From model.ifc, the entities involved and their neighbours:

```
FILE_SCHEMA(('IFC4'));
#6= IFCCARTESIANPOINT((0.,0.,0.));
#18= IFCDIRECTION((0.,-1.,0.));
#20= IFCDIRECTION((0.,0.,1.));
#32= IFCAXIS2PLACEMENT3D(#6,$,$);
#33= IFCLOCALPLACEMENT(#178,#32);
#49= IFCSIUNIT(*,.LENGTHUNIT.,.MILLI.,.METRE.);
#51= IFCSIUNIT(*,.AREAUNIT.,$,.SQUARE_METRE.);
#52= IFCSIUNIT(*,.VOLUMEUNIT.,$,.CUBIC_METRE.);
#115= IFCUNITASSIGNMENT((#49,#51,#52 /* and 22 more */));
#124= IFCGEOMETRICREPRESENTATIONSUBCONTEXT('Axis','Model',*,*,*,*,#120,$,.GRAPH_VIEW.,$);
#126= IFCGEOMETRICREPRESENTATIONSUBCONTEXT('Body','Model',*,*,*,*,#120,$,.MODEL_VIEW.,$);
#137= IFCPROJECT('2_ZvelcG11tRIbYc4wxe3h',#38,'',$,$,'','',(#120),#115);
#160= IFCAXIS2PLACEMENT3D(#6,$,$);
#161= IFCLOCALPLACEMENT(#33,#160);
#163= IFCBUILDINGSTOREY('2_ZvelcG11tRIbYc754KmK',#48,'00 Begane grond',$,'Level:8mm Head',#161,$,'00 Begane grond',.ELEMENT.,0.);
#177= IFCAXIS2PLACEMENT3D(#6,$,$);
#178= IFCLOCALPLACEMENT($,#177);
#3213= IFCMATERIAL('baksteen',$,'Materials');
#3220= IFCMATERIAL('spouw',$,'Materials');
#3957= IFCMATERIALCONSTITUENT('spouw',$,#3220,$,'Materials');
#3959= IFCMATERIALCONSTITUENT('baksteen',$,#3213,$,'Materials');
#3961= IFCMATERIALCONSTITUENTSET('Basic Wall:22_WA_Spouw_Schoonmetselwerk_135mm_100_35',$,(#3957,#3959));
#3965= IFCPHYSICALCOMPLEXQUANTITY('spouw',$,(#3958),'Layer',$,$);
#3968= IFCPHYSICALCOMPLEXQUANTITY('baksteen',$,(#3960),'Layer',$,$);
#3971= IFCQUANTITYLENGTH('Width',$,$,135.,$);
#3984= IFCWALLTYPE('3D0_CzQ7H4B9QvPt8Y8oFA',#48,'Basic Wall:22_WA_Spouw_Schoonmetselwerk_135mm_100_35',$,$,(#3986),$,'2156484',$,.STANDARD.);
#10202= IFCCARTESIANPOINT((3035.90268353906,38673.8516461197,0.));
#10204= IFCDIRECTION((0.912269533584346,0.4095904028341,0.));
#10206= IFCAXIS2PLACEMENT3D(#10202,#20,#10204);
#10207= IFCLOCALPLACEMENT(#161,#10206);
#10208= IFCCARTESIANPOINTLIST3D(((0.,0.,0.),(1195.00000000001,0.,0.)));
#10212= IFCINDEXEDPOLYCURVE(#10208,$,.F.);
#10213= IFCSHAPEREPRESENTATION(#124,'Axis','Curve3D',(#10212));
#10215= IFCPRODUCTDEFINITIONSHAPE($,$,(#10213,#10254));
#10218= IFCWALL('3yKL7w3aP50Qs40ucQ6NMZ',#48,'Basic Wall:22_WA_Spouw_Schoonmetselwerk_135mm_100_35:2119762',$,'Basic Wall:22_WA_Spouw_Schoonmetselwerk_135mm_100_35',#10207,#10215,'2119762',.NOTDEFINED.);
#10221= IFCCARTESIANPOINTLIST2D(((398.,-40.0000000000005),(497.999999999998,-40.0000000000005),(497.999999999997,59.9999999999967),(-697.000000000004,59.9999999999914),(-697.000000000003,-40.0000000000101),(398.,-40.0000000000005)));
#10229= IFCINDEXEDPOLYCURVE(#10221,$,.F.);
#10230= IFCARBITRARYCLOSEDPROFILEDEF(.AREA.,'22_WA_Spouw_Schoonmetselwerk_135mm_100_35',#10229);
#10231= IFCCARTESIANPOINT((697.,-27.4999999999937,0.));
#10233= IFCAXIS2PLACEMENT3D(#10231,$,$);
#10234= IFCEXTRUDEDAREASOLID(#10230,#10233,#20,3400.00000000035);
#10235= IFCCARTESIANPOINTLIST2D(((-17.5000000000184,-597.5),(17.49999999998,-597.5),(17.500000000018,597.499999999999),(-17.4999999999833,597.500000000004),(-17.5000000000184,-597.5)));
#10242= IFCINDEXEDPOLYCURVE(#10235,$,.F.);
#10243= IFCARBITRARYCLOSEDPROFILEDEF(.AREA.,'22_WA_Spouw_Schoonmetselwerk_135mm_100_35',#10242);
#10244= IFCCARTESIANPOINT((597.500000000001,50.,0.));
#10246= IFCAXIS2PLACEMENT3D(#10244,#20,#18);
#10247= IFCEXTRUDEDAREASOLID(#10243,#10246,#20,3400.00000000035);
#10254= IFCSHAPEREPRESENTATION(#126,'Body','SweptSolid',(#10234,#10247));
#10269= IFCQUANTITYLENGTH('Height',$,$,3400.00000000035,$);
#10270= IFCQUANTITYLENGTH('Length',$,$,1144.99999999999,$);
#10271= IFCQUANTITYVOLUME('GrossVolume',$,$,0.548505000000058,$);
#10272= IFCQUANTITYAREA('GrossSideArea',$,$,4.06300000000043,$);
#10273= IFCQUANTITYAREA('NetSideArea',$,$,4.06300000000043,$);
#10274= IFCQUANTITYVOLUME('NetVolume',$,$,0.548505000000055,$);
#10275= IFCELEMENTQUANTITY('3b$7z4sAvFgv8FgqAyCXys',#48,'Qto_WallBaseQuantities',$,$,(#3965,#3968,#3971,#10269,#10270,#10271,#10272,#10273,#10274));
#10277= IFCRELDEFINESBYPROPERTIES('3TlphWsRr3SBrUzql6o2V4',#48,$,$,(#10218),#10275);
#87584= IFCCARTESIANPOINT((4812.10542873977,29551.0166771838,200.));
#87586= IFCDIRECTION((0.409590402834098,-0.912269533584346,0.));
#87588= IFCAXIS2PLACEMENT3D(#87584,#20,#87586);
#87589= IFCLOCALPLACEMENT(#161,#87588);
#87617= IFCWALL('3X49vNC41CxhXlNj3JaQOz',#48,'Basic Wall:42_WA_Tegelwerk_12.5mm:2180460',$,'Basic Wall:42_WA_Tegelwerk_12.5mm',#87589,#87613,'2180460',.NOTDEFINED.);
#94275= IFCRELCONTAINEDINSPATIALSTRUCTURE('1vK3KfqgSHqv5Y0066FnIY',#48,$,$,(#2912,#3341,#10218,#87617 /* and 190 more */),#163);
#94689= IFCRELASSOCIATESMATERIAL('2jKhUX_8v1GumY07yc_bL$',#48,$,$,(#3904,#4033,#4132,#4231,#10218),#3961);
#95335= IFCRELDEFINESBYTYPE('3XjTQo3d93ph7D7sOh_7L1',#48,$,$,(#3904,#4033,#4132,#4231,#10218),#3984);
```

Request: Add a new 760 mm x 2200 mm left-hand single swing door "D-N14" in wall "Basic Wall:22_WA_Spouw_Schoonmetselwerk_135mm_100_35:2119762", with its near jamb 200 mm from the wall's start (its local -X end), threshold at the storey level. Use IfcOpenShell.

```python
import numpy as np
import ifcopenshell
import ifcopenshell.api.feature
import ifcopenshell.api.geometry
import ifcopenshell.api.pset
import ifcopenshell.api.root
import ifcopenshell.api.spatial
import ifcopenshell.geom
import ifcopenshell.util.element
import ifcopenshell.util.placement
import ifcopenshell.util.representation
import ifcopenshell.util.shape
import ifcopenshell.util.unit

model = ifcopenshell.open("model.ifc")
unit_scale = ifcopenshell.util.unit.calculate_unit_scale(model)
area_scale = ifcopenshell.util.unit.calculate_unit_scale(model, "AREAUNIT")
volume_scale = ifcopenshell.util.unit.calculate_unit_scale(model, "VOLUMEUNIT")
settings = ifcopenshell.geom.settings()


def volume(element):
    """Net volume in cubic metres, openings subtracted."""
    shape = ifcopenshell.geom.create_shape(settings, element)
    return ifcopenshell.util.shape.get_volume(shape.geometry)


wall = model.by_guid("3yKL7w3aP50Qs40ucQ6NMZ")
storey = ifcopenshell.util.element.get_container(wall, ifc_class="IfcBuildingStorey")
context = ifcopenshell.util.representation.get_context(model, "Model", "Body", "MODEL_VIEW")
before = volume(wall)

width, height, from_end, sill = 0.76, 2.2, 0.2, 0.0  # metres

# The wall runs along its own X axis, and the end named is its -X end.
wall_shape = ifcopenshell.geom.create_shape(settings, wall)
x, y, z = ifcopenshell.util.shape.get_vertices(wall_shape.geometry).T
start = x.min() + from_end
face, thickness = float(y.min()), float(y.max() - y.min())
wall_matrix = ifcopenshell.util.placement.get_local_placement(wall.ObjectPlacement)
level = ifcopenshell.util.placement.get_local_placement(storey.ObjectPlacement)[2, 3]


def in_wall(x, y):
    """Placement at x, y metres in the wall's axes, at sill height."""
    matrix = wall_matrix.copy()
    matrix[:, 3] = wall_matrix @ np.array([x / unit_scale, y / unit_scale, 0.0, 1.0])
    matrix[2, 3] = level + sill / unit_scale
    return matrix


# Opening: a box that overshoots both wall faces by 50 mm.
opening = ifcopenshell.api.root.create_entity(model, ifc_class="IfcOpeningElement", predefined_type="OPENING")
box = ifcopenshell.api.geometry.add_wall_representation(
    model, context=context, length=width, height=height, thickness=thickness + 0.1
)
ifcopenshell.api.geometry.assign_representation(model, product=opening, representation=box)
ifcopenshell.api.geometry.edit_object_placement(model, product=opening, matrix=in_wall(start, face - 0.05), is_si=False)
ifcopenshell.api.feature.add_feature(model, feature=opening, element=wall)

door = ifcopenshell.api.root.create_entity(model, ifc_class="IfcDoor", name="D-N14", predefined_type="DOOR")
door.OverallWidth, door.OverallHeight = width / unit_scale, height / unit_scale
door.OperationType = "SINGLE_SWING_LEFT"
body = ifcopenshell.api.geometry.add_door_representation(
    model,
    context=context,
    overall_width=door.OverallWidth,
    overall_height=door.OverallHeight,
    operation_type="SINGLE_SWING_LEFT",
    lining_properties={"LiningDepth": thickness / unit_scale, "ThresholdDepth": thickness / unit_scale},
)
ifcopenshell.api.geometry.assign_representation(model, product=door, representation=body)
ifcopenshell.api.spatial.assign_container(model, products=[door], relating_structure=storey)
ifcopenshell.api.feature.add_filling(model, opening=opening, element=door)

# The lining spans the wall, so the door starts at the wall face.
ifcopenshell.api.geometry.edit_object_placement(model, product=door, matrix=in_wall(start, face), is_si=False)

after = volume(wall)

# Update the wall's stored quantities.
qto = model.by_id(ifcopenshell.util.element.get_pset(wall, "Qto_WallBaseQuantities", should_inherit=False)["id"])
ifcopenshell.api.pset.edit_qto(model, qto=qto, properties={
    "NetSideArea": after / thickness / area_scale,
    "NetVolume": after / volume_scale,
})

print(f"wall volume {before:.3f} -> {after:.3f} m3")

model.write("model-out.ifc")
```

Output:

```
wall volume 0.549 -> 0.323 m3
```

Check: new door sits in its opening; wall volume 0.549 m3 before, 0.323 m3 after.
